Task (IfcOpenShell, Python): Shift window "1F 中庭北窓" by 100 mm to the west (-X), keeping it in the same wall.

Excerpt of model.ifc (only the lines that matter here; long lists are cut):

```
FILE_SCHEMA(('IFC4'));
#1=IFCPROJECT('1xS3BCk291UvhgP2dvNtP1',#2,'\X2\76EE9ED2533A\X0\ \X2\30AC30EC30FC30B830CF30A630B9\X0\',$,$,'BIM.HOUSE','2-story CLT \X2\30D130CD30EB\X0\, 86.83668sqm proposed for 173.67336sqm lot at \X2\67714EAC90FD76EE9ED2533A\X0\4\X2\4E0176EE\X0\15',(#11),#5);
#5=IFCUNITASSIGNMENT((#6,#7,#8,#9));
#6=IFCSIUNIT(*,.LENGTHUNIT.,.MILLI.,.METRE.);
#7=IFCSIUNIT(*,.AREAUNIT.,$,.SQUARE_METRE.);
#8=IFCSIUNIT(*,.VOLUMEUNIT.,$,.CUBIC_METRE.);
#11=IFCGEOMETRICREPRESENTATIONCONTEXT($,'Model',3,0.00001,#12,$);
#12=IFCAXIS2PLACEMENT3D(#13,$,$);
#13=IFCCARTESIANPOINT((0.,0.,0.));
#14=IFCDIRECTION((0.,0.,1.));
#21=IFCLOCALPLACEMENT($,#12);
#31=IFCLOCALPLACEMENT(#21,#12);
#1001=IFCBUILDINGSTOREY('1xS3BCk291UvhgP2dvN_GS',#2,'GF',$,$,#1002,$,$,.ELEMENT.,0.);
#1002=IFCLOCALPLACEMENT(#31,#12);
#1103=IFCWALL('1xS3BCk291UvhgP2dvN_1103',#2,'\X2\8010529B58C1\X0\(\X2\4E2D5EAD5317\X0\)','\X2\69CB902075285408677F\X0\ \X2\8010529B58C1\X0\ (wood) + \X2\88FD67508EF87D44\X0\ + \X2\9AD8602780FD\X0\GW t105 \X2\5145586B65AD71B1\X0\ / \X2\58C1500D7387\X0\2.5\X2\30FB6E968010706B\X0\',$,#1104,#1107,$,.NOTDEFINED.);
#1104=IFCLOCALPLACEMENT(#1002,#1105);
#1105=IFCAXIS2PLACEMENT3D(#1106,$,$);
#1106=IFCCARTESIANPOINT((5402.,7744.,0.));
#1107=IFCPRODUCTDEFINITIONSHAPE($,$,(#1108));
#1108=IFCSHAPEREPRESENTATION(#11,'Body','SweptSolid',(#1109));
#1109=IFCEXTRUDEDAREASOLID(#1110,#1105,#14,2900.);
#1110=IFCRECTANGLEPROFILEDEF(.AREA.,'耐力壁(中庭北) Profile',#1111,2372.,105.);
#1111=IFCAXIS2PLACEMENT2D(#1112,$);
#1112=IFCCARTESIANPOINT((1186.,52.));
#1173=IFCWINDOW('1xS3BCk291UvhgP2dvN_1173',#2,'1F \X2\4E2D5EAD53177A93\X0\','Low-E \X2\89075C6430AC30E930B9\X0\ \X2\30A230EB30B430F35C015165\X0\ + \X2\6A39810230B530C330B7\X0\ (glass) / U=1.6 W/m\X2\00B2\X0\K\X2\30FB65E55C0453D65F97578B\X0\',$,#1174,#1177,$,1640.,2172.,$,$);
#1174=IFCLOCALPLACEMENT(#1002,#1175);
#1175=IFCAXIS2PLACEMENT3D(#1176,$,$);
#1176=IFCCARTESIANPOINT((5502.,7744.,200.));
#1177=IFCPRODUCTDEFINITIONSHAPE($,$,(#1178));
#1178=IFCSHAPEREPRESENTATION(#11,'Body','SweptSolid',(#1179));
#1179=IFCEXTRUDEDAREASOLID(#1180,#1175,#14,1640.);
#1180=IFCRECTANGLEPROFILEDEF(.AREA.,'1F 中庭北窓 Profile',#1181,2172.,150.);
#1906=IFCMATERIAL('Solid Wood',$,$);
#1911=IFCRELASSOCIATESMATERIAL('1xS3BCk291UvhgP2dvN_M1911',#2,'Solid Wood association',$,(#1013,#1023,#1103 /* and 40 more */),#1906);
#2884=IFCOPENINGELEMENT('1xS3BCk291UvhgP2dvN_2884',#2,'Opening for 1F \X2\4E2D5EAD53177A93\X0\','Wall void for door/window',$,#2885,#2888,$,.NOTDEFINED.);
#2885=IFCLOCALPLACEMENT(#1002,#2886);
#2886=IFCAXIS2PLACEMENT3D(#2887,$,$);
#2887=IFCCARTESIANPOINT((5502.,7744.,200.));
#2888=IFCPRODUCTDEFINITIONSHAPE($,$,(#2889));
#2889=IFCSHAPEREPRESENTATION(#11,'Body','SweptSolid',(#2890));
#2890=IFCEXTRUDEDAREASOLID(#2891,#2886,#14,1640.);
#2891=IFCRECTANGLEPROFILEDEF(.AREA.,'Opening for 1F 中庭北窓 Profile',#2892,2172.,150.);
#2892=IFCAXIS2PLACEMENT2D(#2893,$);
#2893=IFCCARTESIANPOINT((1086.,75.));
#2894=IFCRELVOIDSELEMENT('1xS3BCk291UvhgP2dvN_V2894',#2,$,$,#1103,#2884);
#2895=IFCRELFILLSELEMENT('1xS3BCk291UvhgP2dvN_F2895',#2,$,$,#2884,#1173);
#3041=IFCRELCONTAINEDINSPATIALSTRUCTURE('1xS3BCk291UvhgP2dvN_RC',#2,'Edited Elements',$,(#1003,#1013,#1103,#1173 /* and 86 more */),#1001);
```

```python
import ifcopenshell
import ifcopenshell.api.geometry
import ifcopenshell.util.placement

model = ifcopenshell.open("model.ifc")

window = model.by_guid("1xS3BCk291UvhgP2dvN_1173")
opening = window.FillsVoids[0].RelatingOpeningElement
wall = opening.VoidsElements[0].RelatingBuildingElement

wall_matrix = ifcopenshell.util.placement.get_local_placement(wall.ObjectPlacement)
shift = wall_matrix[:3, 0] * -100.0
before = ifcopenshell.util.placement.get_local_placement(window.ObjectPlacement)[:3, 3].copy()

# The window is not placed relative to its opening, so move both.
for product in (opening, window):
    matrix = ifcopenshell.util.placement.get_local_placement(product.ObjectPlacement)
    matrix[:3, 3] += shift
    ifcopenshell.api.geometry.edit_object_placement(model, product=product, matrix=matrix, is_si=False)

after = ifcopenshell.util.placement.get_local_placement(window.ObjectPlacement)[:3, 3]
print("window moved by", (after - before).round(3) + 0.0)

model.write("model_updated.ifc")
```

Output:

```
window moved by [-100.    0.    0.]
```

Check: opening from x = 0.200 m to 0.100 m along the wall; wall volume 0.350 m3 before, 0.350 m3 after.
